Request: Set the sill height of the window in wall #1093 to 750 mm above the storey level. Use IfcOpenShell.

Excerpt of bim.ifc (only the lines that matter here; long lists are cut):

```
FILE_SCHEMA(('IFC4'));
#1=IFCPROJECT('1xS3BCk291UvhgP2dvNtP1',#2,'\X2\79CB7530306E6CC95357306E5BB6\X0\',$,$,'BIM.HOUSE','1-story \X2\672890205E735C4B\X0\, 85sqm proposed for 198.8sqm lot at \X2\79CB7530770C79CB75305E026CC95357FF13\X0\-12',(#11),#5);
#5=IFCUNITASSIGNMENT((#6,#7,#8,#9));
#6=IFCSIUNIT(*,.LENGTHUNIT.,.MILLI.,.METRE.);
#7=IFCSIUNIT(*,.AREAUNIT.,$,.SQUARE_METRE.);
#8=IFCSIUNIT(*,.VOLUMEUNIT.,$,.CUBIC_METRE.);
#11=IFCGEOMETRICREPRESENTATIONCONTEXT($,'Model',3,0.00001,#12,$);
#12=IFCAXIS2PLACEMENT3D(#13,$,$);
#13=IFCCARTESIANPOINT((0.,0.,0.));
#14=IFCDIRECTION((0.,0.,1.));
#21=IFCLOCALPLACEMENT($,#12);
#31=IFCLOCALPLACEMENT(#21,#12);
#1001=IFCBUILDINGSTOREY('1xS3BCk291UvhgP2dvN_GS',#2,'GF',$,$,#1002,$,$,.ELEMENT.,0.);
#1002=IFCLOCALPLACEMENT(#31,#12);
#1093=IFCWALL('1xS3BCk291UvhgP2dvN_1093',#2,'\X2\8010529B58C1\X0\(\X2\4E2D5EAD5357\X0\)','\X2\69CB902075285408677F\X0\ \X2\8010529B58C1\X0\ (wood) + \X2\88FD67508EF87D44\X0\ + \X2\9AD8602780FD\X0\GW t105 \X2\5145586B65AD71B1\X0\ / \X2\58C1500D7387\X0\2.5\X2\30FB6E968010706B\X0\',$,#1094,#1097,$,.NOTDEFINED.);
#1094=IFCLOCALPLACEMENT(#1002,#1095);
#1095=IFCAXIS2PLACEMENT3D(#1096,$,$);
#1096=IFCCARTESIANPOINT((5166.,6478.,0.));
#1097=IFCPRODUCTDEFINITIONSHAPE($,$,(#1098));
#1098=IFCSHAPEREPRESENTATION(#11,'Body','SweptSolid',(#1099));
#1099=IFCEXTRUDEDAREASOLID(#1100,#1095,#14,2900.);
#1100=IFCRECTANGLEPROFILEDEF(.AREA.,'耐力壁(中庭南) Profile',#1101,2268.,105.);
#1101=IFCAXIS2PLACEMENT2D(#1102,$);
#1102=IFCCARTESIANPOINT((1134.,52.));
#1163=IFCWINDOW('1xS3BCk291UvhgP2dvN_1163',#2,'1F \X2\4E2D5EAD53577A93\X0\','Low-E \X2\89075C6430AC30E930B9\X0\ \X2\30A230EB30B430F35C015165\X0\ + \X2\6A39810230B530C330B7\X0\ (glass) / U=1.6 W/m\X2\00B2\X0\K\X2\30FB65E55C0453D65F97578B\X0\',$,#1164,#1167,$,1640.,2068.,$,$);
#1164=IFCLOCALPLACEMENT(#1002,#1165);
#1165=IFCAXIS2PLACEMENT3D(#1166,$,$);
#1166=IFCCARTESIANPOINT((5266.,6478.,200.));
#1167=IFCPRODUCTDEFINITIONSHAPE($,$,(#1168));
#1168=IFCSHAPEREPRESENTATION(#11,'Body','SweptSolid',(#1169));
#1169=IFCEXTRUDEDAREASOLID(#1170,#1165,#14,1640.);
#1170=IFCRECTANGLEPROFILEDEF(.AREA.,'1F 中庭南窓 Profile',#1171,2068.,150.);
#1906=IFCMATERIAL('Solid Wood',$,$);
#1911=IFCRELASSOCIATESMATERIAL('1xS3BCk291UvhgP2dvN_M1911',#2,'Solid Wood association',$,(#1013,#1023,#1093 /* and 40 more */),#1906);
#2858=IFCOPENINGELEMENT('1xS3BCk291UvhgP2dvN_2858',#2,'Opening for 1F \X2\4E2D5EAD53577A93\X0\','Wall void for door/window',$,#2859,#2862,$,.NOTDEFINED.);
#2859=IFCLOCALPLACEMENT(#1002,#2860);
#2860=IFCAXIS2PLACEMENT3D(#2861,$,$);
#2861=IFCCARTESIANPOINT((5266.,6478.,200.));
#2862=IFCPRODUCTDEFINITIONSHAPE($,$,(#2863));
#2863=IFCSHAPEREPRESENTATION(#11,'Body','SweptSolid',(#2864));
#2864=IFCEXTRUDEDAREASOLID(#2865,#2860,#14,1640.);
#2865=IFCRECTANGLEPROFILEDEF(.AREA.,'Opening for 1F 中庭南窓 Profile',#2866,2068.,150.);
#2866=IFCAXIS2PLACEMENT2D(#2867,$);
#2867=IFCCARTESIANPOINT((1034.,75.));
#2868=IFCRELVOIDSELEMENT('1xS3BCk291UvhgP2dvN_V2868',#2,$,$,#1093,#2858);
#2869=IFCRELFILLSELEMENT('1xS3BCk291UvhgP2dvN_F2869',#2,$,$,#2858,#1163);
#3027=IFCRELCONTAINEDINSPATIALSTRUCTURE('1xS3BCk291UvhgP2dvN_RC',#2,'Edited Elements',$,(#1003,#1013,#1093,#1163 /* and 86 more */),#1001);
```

```python
import numpy as np
import ifcopenshell
import ifcopenshell.api.geometry
import ifcopenshell.geom
import ifcopenshell.util.element
import ifcopenshell.util.placement
import ifcopenshell.util.shape
import ifcopenshell.util.unit

model = ifcopenshell.open("bim.ifc")
unit_scale = ifcopenshell.util.unit.calculate_unit_scale(model)

window = model.by_guid("1xS3BCk291UvhgP2dvN_1163")
opening = window.FillsVoids[0].RelatingOpeningElement
storey = ifcopenshell.util.element.get_container(window, ifc_class="IfcBuildingStorey")
level = ifcopenshell.util.placement.get_local_placement(storey.ObjectPlacement)[2, 3]

# The opening's origin need not be at the sill, so measure its lowest point.
shape = ifcopenshell.geom.create_shape(ifcopenshell.geom.settings(), opening)
bottom = ifcopenshell.util.shape.get_shape_bottom_elevation(shape, shape.geometry) / unit_scale
dz = level + 0.75 / unit_scale - bottom

shift = np.array([0.0, 0.0, dz])
# The window is not placed relative to its opening, so move both.
for product in (opening, window):
    matrix = ifcopenshell.util.placement.get_local_placement(product.ObjectPlacement)
    matrix[:3, 3] += shift
    ifcopenshell.api.geometry.edit_object_placement(model, product=product, matrix=matrix, is_si=False)

print(f"moved by {dz * unit_scale:+.3f} m")

model.write("bim_v2.ifc")
```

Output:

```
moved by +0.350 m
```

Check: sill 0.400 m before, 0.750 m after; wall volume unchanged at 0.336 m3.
